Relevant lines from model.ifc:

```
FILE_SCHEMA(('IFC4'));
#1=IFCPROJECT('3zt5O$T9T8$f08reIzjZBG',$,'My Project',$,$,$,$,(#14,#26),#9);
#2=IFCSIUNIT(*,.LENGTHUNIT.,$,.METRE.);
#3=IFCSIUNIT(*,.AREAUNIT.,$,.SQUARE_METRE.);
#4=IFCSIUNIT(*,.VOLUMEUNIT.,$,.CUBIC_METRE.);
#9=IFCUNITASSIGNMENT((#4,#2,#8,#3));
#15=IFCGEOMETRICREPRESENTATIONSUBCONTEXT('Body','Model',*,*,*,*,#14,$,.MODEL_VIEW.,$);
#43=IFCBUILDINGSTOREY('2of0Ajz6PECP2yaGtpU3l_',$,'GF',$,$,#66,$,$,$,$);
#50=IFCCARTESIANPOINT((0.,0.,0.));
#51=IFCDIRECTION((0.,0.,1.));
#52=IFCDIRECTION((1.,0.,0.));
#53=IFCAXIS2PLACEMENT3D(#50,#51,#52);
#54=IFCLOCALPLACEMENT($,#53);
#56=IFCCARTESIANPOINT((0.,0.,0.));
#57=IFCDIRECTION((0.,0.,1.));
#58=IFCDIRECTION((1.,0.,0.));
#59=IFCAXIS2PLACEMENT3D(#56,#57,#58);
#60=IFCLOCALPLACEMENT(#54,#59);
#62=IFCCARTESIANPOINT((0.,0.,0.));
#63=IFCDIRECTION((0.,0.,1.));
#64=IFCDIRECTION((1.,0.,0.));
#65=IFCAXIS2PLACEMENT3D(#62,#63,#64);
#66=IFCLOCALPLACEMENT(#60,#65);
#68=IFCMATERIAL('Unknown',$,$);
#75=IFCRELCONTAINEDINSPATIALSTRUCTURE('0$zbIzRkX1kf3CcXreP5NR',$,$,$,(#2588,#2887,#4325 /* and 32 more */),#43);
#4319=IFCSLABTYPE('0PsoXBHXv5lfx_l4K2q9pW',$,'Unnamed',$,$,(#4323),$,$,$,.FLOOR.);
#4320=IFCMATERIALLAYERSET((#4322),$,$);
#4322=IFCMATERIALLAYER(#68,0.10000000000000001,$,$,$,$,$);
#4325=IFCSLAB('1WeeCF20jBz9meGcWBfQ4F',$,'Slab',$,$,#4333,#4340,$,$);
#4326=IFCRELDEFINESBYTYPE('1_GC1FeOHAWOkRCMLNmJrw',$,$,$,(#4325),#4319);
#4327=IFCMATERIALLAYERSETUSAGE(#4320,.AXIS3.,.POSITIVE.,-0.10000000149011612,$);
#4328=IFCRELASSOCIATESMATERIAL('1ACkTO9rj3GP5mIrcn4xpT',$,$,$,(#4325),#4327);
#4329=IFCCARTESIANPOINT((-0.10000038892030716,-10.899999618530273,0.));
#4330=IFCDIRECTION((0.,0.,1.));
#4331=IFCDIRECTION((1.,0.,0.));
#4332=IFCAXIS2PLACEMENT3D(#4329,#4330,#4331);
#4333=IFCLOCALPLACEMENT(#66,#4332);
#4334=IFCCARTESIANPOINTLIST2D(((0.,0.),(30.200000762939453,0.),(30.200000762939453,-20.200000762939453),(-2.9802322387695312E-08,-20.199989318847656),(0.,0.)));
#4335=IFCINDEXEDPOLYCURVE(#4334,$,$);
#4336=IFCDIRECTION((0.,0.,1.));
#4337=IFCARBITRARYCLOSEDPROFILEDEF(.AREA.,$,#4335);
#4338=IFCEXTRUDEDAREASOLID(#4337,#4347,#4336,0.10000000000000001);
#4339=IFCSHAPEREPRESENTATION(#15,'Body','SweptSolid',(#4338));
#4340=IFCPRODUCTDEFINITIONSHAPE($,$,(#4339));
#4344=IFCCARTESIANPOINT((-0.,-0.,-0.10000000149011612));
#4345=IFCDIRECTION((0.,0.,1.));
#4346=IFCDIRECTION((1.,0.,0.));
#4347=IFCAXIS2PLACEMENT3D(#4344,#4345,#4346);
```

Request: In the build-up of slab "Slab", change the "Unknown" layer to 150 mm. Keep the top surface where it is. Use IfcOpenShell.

```python
import ifcopenshell
import ifcopenshell.util.element
import ifcopenshell.util.representation

model = ifcopenshell.open("model.ifc")

layer_set = model.by_id(4320)
layer = next(l for l in layer_set.MaterialLayers if l.Material and l.Material.Name == "Unknown")
change = 0.15 - layer.LayerThickness
layer.LayerThickness += change

# Geometry does not follow the layer set by itself.
slabs = [e for e in ifcopenshell.util.element.get_elements_by_material(model, layer_set) if e.is_a("IfcSlab")]
for slab in sorted(slabs, key=lambda e: e.id()):
    body = ifcopenshell.util.representation.get_representation(slab, "Model", "Body")
    solid = body.Items[0]
    old_depth = solid.Depth
    solid.Depth += change
    # Extruded upwards: lower the start of the extrusion so the top stays.
    x, y, z = solid.Position.Location.Coordinates
    solid.Position.Location = model.createIfcCartesianPoint((x, y, z - change))
    print(slab.id(), f"{old_depth:g} -> {solid.Depth:g}")

# The layers are counted up from the underside, which has moved.
for usage in {ifcopenshell.util.element.get_material(slab) for slab in slabs}:
    usage.OffsetFromReferenceLine -= change

model.write("model_rev.ifc")
```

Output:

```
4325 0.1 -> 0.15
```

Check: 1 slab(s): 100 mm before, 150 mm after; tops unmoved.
